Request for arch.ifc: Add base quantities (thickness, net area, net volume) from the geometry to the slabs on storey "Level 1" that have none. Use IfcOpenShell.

First a look at what the model holds.

```python
import ifcopenshell
import ifcopenshell.util.element
import ifcopenshell.util.unit

model = ifcopenshell.open("arch.ifc")
print(model.schema)
for unit_type in ("LENGTHUNIT", "AREAUNIT", "VOLUMEUNIT"):
    print(unit_type, ifcopenshell.util.unit.calculate_unit_scale(model, unit_type))
storey = next(s for s in model.by_type("IfcBuildingStorey") if s.Name == "Level 1")
slabs = [e for e in ifcopenshell.util.element.get_decomposition(storey) if e.is_a("IfcSlab")]
for e in sorted(slabs, key=lambda e: e.id()):
    print(e.id(), e.is_a(), e.Name, list(ifcopenshell.util.element.get_psets(e, qtos_only=True)), sep=" | ")
```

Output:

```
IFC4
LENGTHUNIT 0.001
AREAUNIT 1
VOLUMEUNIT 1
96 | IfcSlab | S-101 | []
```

```python
import ifcopenshell
import ifcopenshell.api.pset
import ifcopenshell.geom
import ifcopenshell.util.element
import ifcopenshell.util.shape
import ifcopenshell.util.unit

model = ifcopenshell.open("arch.ifc")
unit_scale = ifcopenshell.util.unit.calculate_unit_scale(model)
area_scale = ifcopenshell.util.unit.calculate_unit_scale(model, "AREAUNIT")
volume_scale = ifcopenshell.util.unit.calculate_unit_scale(model, "VOLUMEUNIT")
settings = ifcopenshell.geom.settings()

storey = next(s for s in model.by_type("IfcBuildingStorey") if s.Name == "Level 1")
slabs = [e for e in ifcopenshell.util.element.get_decomposition(storey) if e.is_a("IfcSlab")]

for e in sorted(slabs, key=lambda e: e.id()):
    if ifcopenshell.util.element.get_psets(e, qtos_only=True, should_inherit=False):
        continue
    # Geometry comes back in metres, in the element's own axes.
    shape = ifcopenshell.geom.create_shape(settings, e)
    values = {
        "Width": ifcopenshell.util.shape.get_z(shape.geometry) / unit_scale,
        "NetArea": ifcopenshell.util.shape.get_footprint_area(shape.geometry) / area_scale,
        "NetVolume": ifcopenshell.util.shape.get_volume(shape.geometry) / volume_scale,
    }
    qto = ifcopenshell.api.pset.add_qto(model, product=e, name="Qto_SlabBaseQuantities")
    ifcopenshell.api.pset.edit_qto(model, qto=qto, properties=values)
    print(e.id(), {k: round(v, 3) for k, v in values.items()})

model.write("arch_v2.ifc")
```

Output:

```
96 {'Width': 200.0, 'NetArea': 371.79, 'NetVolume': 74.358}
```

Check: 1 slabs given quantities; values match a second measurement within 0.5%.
